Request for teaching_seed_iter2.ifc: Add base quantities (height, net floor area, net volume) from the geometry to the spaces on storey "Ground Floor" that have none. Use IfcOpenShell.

First a look at what the model holds.

```python
import ifcopenshell
import ifcopenshell.util.element
import ifcopenshell.util.unit

model = ifcopenshell.open("teaching_seed_iter2.ifc")
print(model.schema)
for unit_type in ("LENGTHUNIT", "AREAUNIT", "VOLUMEUNIT"):
    print(unit_type, ifcopenshell.util.unit.calculate_unit_scale(model, unit_type))
storey = next(s for s in model.by_type("IfcBuildingStorey") if s.Name == "Ground Floor")
spaces = [e for e in ifcopenshell.util.element.get_decomposition(storey) if e.is_a("IfcSpace")]
for e in sorted(spaces, key=lambda e: e.id()):
    print(e.id(), e.is_a(), e.Name, list(ifcopenshell.util.element.get_psets(e, qtos_only=True)), sep=" | ")
```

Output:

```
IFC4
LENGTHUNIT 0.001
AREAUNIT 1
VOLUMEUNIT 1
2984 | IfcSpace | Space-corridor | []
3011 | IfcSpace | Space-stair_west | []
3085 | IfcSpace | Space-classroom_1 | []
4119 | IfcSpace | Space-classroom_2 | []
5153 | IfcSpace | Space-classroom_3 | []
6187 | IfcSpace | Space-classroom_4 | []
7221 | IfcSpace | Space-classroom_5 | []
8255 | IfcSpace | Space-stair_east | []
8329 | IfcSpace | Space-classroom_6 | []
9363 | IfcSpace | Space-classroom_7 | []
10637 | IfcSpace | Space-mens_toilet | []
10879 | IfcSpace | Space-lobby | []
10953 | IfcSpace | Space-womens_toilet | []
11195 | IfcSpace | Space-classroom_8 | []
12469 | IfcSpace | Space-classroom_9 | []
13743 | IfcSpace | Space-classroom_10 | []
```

```python
import ifcopenshell
import ifcopenshell.api.pset
import ifcopenshell.geom
import ifcopenshell.util.element
import ifcopenshell.util.shape
import ifcopenshell.util.unit

model = ifcopenshell.open("teaching_seed_iter2.ifc")
unit_scale = ifcopenshell.util.unit.calculate_unit_scale(model)
area_scale = ifcopenshell.util.unit.calculate_unit_scale(model, "AREAUNIT")
volume_scale = ifcopenshell.util.unit.calculate_unit_scale(model, "VOLUMEUNIT")
settings = ifcopenshell.geom.settings()

storey = next(s for s in model.by_type("IfcBuildingStorey") if s.Name == "Ground Floor")
spaces = [e for e in ifcopenshell.util.element.get_decomposition(storey) if e.is_a("IfcSpace")]

for e in sorted(spaces, key=lambda e: e.id()):
    if ifcopenshell.util.element.get_psets(e, qtos_only=True, should_inherit=False):
        continue
    # Geometry comes back in metres, in the element's own axes.
    shape = ifcopenshell.geom.create_shape(settings, e)
    values = {
        "Height": ifcopenshell.util.shape.get_z(shape.geometry) / unit_scale,
        "NetFloorArea": ifcopenshell.util.shape.get_footprint_area(shape.geometry) / area_scale,
        "NetVolume": ifcopenshell.util.shape.get_volume(shape.geometry) / volume_scale,
    }
    qto = ifcopenshell.api.pset.add_qto(model, product=e, name="Qto_SpaceBaseQuantities")
    ifcopenshell.api.pset.edit_qto(model, qto=qto, properties=values)
    print(e.id(), {k: round(v, 3) for k, v in values.items()})

model.write("teaching_seed_iter2_rev.ifc")
```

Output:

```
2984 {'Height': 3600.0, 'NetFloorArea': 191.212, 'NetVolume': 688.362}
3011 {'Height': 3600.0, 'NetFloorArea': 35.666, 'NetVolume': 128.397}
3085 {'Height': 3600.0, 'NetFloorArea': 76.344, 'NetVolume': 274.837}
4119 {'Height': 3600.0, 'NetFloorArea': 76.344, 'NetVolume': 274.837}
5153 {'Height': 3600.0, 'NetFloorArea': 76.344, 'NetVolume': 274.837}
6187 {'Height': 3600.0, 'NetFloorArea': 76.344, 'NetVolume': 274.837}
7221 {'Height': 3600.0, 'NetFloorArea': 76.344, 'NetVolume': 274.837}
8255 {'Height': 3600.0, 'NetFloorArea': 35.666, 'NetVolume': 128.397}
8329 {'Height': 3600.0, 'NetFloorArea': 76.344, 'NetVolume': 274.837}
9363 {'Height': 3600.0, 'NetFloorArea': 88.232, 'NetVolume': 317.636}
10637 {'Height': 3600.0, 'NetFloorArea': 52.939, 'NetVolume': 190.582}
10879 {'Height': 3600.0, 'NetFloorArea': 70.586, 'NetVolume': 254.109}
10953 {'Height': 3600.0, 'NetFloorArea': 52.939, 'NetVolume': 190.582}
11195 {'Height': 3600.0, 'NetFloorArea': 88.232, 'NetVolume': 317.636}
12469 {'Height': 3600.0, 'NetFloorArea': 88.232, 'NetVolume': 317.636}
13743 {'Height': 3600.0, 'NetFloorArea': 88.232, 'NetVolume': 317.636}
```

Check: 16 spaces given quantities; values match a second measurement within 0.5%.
